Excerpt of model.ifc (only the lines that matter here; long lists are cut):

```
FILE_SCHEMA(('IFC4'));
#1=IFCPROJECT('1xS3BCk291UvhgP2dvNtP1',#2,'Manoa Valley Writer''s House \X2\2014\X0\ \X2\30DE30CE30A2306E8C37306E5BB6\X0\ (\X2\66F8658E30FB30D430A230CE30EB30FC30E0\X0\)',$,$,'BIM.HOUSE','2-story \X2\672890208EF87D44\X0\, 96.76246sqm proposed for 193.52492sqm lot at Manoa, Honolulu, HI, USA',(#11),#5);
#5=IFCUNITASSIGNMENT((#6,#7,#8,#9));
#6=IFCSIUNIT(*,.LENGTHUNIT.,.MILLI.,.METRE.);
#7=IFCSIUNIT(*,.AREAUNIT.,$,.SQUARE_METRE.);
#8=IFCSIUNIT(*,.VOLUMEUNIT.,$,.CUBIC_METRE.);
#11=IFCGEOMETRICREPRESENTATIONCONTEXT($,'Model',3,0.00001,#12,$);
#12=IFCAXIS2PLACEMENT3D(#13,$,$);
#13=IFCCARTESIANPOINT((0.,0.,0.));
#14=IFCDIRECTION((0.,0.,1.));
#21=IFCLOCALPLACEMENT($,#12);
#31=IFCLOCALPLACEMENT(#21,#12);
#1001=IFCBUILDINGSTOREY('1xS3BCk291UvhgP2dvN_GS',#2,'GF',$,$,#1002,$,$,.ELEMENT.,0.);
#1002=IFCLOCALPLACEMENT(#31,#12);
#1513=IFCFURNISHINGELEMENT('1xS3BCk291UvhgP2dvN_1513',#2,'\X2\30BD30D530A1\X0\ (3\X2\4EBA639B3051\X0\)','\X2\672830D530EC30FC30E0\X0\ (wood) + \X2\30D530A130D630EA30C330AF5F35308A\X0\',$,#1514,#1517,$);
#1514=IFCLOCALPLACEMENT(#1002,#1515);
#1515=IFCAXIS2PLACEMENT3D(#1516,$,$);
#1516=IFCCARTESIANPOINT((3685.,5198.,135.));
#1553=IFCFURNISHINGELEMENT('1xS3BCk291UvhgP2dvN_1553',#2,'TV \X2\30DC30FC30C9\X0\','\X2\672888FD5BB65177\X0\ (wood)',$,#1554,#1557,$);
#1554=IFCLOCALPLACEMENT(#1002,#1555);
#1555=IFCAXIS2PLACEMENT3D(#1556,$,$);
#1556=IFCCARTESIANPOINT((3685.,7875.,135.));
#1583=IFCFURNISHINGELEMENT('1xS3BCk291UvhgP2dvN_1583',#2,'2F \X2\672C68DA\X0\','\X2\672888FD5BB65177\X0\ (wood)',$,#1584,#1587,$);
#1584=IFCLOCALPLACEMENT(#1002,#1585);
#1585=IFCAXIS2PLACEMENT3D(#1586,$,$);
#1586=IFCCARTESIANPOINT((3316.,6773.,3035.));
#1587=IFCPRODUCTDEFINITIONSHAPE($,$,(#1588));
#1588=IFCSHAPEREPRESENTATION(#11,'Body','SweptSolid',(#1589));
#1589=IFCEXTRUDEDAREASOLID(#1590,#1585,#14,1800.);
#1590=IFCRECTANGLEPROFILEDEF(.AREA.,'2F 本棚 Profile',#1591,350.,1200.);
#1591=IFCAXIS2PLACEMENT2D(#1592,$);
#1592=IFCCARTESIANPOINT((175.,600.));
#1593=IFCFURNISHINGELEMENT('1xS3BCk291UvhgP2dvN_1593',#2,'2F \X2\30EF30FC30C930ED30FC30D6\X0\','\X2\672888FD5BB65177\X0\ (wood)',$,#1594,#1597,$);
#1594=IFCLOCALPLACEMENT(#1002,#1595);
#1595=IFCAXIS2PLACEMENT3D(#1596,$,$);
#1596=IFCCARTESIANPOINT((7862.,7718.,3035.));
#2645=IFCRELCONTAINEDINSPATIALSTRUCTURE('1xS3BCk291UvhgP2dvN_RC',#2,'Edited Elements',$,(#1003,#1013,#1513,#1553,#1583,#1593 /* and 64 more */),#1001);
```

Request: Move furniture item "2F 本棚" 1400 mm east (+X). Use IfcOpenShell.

```python
import ifcopenshell
import ifcopenshell.api.geometry
import ifcopenshell.util.placement

model = ifcopenshell.open("model.ifc")

item = model.by_guid("1xS3BCk291UvhgP2dvN_1583")
matrix = ifcopenshell.util.placement.get_local_placement(item.ObjectPlacement)
matrix[0, 3] += 1400.0
ifcopenshell.api.geometry.edit_object_placement(model, product=item, matrix=matrix, is_si=False)

print(ifcopenshell.util.placement.get_local_placement(item.ObjectPlacement).round(3) + 0.0)

model.write("model_v2.ifc")
```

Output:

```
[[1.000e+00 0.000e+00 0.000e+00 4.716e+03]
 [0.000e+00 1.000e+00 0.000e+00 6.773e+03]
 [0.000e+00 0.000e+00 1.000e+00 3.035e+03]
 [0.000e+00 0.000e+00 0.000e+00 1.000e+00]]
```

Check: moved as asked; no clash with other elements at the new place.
